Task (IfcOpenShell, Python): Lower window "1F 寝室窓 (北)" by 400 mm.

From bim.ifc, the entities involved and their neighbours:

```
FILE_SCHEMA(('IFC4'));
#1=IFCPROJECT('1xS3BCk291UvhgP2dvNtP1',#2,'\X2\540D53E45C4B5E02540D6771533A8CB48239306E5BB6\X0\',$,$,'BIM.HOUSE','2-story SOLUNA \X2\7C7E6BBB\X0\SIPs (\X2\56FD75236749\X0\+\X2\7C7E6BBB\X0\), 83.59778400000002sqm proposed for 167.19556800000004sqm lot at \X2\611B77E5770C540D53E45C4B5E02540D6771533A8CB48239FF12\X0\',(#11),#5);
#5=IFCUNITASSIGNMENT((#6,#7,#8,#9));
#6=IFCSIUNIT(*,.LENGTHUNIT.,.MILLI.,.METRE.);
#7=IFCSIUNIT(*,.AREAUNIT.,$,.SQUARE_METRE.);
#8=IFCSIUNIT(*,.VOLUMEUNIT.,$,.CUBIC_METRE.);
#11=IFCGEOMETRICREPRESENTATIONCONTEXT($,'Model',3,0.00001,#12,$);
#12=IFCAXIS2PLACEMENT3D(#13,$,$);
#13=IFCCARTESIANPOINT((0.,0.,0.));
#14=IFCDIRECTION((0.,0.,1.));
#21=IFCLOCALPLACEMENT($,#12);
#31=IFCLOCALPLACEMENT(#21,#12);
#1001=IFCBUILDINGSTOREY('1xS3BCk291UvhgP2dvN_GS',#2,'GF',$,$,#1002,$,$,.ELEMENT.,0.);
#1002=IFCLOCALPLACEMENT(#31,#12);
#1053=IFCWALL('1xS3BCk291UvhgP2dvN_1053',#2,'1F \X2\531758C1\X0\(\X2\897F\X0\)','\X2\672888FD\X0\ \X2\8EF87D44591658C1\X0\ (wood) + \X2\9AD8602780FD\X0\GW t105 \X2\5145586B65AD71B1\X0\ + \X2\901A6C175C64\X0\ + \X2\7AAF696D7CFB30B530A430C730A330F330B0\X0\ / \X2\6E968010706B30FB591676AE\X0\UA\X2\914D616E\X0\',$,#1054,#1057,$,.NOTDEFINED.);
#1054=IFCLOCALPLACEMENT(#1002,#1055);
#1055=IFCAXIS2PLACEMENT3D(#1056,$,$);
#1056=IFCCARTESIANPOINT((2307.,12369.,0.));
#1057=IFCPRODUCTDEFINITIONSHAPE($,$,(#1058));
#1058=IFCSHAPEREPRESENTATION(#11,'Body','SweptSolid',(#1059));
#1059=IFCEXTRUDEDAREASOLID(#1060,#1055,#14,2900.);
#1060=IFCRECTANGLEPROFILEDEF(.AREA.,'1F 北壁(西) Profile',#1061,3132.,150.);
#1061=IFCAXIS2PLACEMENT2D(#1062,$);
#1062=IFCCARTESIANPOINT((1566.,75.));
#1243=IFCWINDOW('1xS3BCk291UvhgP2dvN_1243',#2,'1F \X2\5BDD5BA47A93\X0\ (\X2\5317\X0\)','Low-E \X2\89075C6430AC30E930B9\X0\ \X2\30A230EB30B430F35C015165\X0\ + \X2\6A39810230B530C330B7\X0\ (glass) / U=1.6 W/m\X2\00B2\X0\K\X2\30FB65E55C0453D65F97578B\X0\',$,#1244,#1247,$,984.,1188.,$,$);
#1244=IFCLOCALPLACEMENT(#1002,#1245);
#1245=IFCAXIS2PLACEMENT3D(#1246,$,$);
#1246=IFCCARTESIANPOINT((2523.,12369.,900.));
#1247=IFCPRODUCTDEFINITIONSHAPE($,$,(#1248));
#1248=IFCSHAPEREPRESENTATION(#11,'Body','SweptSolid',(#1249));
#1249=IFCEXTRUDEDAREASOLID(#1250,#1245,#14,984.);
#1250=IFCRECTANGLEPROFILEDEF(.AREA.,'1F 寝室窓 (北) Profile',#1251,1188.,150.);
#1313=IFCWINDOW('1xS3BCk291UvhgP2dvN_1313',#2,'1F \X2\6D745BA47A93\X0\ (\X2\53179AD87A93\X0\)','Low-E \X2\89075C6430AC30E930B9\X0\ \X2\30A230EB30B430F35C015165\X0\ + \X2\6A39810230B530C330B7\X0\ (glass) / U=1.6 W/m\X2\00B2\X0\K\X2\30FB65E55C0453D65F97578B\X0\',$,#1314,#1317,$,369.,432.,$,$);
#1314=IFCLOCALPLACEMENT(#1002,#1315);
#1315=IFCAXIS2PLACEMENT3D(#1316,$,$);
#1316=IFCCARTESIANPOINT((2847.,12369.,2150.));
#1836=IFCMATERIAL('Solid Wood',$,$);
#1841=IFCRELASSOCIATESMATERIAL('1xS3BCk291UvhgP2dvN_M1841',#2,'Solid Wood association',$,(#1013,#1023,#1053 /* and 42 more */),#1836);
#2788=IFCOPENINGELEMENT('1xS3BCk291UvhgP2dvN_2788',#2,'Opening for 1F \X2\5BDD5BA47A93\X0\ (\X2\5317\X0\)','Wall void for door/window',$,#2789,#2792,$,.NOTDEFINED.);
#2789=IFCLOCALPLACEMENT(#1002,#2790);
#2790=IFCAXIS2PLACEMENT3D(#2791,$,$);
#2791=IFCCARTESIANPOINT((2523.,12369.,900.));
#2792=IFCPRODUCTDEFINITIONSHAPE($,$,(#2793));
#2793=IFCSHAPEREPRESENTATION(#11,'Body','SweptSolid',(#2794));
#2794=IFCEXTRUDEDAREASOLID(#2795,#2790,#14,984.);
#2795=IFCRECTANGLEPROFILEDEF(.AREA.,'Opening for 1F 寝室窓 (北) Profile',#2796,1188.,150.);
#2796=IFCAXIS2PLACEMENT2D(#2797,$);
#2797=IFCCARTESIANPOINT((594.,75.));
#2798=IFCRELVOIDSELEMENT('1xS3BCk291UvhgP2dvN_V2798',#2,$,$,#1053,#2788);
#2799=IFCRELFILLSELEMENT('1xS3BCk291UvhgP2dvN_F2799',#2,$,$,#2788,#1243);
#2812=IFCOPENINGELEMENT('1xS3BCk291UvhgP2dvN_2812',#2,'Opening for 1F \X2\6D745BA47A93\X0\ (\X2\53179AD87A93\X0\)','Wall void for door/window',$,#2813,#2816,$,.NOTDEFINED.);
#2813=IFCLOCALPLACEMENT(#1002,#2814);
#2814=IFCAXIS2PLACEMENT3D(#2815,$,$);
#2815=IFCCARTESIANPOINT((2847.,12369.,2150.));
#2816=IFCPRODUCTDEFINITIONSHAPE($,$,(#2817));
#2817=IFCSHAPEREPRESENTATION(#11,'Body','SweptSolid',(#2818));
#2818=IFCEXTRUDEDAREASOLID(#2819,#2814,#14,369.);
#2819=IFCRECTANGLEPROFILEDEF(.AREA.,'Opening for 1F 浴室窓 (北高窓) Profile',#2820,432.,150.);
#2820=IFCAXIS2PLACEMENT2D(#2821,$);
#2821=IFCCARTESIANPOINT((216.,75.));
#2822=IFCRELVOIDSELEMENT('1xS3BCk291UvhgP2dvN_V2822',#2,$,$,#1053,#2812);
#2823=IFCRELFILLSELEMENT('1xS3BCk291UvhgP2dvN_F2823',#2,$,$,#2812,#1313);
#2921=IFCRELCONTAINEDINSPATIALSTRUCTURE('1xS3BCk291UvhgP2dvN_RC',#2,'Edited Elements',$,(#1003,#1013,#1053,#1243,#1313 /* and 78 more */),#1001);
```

```python
import numpy as np
import ifcopenshell
import ifcopenshell.api.geometry
import ifcopenshell.util.placement
import ifcopenshell.util.unit

model = ifcopenshell.open("bim.ifc")
unit_scale = ifcopenshell.util.unit.calculate_unit_scale(model)

window = model.by_id(1243)
opening = window.FillsVoids[0].RelatingOpeningElement
dz = -400.0

shift = np.array([0.0, 0.0, dz])
# The window is not placed relative to its opening, so move both.
for product in (opening, window):
    matrix = ifcopenshell.util.placement.get_local_placement(product.ObjectPlacement)
    matrix[:3, 3] += shift
    ifcopenshell.api.geometry.edit_object_placement(model, product=product, matrix=matrix, is_si=False)

print(f"moved by {dz * unit_scale:+.3f} m")

model.write("bim_v2.ifc")
```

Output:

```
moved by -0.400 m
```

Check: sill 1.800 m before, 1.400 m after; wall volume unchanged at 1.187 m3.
